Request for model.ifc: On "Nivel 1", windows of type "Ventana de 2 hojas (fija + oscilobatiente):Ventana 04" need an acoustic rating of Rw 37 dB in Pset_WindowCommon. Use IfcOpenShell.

First a look at what the model holds.

```python
import ifcopenshell
import ifcopenshell.util.element

model = ifcopenshell.open("model.ifc")
print(model.schema)
storey = next(s for s in model.by_type("IfcBuildingStorey") if s.Name == "Nivel 1")
windows = [e for e in ifcopenshell.util.element.get_decomposition(storey) if e.is_a("IfcWindow")]
seen = {}
for e in windows:
    element_type = ifcopenshell.util.element.get_type(e)
    key = (element_type.Name if element_type != e and element_type else None, ifcopenshell.util.element.get_pset(e, "Pset_WindowCommon", "AcousticRating"))
    seen[key] = seen.get(key, 0) + 1
for (name, value), count in sorted(seen.items(), key=str):
    print(count, "x", name, "|", value)
```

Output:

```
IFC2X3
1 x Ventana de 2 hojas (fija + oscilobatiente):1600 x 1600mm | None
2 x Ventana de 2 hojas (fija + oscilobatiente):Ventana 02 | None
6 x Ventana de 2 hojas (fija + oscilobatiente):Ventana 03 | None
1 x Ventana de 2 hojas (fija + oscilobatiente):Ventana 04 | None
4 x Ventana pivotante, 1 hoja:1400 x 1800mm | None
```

```python
import ifcopenshell
import ifcopenshell.api.pset
import ifcopenshell.util.element

model = ifcopenshell.open("model.ifc")

storey = next(s for s in model.by_type("IfcBuildingStorey") if s.Name == "Nivel 1")
windows = [e for e in ifcopenshell.util.element.get_decomposition(storey) if e.is_a("IfcWindow")]

count = 0
for e in windows:
    element_type = ifcopenshell.util.element.get_type(e)
    if element_type in (None, e) or element_type.Name != "Ventana de 2 hojas (fija + oscilobatiente):Ventana 04":
        continue
    # add_pset returns the element's existing set when there is one.
    pset = ifcopenshell.api.pset.add_pset(model, product=e, name="Pset_WindowCommon")
    ifcopenshell.api.pset.edit_pset(model, pset=pset, properties={"AcousticRating": "Rw 37 dB"})
    count += 1

print(count, "windows updated")

model.write("model_edited.ifc")
```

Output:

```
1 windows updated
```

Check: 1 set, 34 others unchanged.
